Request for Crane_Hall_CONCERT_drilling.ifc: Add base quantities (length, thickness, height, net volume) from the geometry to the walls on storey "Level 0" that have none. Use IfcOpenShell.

First a look at what the model holds.

```python
import ifcopenshell
import ifcopenshell.util.element
import ifcopenshell.util.unit

model = ifcopenshell.open("Crane_Hall_CONCERT_drilling.ifc")
print(model.schema)
for unit_type in ("LENGTHUNIT", "AREAUNIT", "VOLUMEUNIT"):
    print(unit_type, ifcopenshell.util.unit.calculate_unit_scale(model, unit_type))
storey = next(s for s in model.by_type("IfcBuildingStorey") if s.Name == "Level 0")
walls = [e for e in ifcopenshell.util.element.get_decomposition(storey) if e.is_a("IfcWall")]
for e in sorted(walls, key=lambda e: e.id()):
    print(e.id(), e.is_a(), e.Name, list(ifcopenshell.util.element.get_psets(e, qtos_only=True)), sep=" | ")
```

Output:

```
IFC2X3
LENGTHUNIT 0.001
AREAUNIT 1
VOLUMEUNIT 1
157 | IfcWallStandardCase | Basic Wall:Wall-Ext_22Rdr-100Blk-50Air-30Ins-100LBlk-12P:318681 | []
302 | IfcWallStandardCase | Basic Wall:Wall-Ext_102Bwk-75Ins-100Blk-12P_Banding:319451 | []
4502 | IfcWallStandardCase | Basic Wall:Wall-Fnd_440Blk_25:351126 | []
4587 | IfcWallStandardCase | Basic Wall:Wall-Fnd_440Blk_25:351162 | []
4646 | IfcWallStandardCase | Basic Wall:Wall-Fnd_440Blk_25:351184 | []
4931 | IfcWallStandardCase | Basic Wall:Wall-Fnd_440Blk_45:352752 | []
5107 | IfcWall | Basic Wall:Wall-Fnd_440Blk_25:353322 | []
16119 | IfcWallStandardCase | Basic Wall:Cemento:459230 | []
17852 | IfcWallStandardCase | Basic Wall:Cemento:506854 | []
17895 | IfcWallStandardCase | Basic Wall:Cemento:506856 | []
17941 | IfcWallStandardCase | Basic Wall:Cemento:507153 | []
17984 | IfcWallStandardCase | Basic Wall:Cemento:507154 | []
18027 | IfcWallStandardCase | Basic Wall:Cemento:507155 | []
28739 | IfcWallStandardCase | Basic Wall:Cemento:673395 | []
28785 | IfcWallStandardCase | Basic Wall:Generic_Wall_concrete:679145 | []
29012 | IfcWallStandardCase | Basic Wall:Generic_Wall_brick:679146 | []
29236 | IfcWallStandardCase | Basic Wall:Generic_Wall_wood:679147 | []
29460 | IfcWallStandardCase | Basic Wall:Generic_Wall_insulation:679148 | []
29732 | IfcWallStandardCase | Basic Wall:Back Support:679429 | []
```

```python
import ifcopenshell
import ifcopenshell.api.pset
import ifcopenshell.geom
import ifcopenshell.util.element
import ifcopenshell.util.shape
import ifcopenshell.util.unit

model = ifcopenshell.open("Crane_Hall_CONCERT_drilling.ifc")
unit_scale = ifcopenshell.util.unit.calculate_unit_scale(model)
volume_scale = ifcopenshell.util.unit.calculate_unit_scale(model, "VOLUMEUNIT")
settings = ifcopenshell.geom.settings()

storey = next(s for s in model.by_type("IfcBuildingStorey") if s.Name == "Level 0")
walls = [e for e in ifcopenshell.util.element.get_decomposition(storey) if e.is_a("IfcWall")]

for e in sorted(walls, key=lambda e: e.id()):
    if ifcopenshell.util.element.get_psets(e, qtos_only=True, should_inherit=False):
        continue
    # Geometry comes back in metres, in the element's own axes.
    shape = ifcopenshell.geom.create_shape(settings, e)
    values = {
        "Length": ifcopenshell.util.shape.get_x(shape.geometry) / unit_scale,
        "Width": ifcopenshell.util.shape.get_y(shape.geometry) / unit_scale,
        "Height": ifcopenshell.util.shape.get_z(shape.geometry) / unit_scale,
        "NetVolume": ifcopenshell.util.shape.get_volume(shape.geometry) / volume_scale,
    }
    qto = ifcopenshell.api.pset.add_qto(model, product=e, name="BaseQuantities")
    ifcopenshell.api.pset.edit_qto(model, qto=qto, properties=values)
    print(e.id(), {k: round(v, 3) for k, v in values.items()})

model.write("Crane_Hall_CONCERT_drilling_edited.ifc")
```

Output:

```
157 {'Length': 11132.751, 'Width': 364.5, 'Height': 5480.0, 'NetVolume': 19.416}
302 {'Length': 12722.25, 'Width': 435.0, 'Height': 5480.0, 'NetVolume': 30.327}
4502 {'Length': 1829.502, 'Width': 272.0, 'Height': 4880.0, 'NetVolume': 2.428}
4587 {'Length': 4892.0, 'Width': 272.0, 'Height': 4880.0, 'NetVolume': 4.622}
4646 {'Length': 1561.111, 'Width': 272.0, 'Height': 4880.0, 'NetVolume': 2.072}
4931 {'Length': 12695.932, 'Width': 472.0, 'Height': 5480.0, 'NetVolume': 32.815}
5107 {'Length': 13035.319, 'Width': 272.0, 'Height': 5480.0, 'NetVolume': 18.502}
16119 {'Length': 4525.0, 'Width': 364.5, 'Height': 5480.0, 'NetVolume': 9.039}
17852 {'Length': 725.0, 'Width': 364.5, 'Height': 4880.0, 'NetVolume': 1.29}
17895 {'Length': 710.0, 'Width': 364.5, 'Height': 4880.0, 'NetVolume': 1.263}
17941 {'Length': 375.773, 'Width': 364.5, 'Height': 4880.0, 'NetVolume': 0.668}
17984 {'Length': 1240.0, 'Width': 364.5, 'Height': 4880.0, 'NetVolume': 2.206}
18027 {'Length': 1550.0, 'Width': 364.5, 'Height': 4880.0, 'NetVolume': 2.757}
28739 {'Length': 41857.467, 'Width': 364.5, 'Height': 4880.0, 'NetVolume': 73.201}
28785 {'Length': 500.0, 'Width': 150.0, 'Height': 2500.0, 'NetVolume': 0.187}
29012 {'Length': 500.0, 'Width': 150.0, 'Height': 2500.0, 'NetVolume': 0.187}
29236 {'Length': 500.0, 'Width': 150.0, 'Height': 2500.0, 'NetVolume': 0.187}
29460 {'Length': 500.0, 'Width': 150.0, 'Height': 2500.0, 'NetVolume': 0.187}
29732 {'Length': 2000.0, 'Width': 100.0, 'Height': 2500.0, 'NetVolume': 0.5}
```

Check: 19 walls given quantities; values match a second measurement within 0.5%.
